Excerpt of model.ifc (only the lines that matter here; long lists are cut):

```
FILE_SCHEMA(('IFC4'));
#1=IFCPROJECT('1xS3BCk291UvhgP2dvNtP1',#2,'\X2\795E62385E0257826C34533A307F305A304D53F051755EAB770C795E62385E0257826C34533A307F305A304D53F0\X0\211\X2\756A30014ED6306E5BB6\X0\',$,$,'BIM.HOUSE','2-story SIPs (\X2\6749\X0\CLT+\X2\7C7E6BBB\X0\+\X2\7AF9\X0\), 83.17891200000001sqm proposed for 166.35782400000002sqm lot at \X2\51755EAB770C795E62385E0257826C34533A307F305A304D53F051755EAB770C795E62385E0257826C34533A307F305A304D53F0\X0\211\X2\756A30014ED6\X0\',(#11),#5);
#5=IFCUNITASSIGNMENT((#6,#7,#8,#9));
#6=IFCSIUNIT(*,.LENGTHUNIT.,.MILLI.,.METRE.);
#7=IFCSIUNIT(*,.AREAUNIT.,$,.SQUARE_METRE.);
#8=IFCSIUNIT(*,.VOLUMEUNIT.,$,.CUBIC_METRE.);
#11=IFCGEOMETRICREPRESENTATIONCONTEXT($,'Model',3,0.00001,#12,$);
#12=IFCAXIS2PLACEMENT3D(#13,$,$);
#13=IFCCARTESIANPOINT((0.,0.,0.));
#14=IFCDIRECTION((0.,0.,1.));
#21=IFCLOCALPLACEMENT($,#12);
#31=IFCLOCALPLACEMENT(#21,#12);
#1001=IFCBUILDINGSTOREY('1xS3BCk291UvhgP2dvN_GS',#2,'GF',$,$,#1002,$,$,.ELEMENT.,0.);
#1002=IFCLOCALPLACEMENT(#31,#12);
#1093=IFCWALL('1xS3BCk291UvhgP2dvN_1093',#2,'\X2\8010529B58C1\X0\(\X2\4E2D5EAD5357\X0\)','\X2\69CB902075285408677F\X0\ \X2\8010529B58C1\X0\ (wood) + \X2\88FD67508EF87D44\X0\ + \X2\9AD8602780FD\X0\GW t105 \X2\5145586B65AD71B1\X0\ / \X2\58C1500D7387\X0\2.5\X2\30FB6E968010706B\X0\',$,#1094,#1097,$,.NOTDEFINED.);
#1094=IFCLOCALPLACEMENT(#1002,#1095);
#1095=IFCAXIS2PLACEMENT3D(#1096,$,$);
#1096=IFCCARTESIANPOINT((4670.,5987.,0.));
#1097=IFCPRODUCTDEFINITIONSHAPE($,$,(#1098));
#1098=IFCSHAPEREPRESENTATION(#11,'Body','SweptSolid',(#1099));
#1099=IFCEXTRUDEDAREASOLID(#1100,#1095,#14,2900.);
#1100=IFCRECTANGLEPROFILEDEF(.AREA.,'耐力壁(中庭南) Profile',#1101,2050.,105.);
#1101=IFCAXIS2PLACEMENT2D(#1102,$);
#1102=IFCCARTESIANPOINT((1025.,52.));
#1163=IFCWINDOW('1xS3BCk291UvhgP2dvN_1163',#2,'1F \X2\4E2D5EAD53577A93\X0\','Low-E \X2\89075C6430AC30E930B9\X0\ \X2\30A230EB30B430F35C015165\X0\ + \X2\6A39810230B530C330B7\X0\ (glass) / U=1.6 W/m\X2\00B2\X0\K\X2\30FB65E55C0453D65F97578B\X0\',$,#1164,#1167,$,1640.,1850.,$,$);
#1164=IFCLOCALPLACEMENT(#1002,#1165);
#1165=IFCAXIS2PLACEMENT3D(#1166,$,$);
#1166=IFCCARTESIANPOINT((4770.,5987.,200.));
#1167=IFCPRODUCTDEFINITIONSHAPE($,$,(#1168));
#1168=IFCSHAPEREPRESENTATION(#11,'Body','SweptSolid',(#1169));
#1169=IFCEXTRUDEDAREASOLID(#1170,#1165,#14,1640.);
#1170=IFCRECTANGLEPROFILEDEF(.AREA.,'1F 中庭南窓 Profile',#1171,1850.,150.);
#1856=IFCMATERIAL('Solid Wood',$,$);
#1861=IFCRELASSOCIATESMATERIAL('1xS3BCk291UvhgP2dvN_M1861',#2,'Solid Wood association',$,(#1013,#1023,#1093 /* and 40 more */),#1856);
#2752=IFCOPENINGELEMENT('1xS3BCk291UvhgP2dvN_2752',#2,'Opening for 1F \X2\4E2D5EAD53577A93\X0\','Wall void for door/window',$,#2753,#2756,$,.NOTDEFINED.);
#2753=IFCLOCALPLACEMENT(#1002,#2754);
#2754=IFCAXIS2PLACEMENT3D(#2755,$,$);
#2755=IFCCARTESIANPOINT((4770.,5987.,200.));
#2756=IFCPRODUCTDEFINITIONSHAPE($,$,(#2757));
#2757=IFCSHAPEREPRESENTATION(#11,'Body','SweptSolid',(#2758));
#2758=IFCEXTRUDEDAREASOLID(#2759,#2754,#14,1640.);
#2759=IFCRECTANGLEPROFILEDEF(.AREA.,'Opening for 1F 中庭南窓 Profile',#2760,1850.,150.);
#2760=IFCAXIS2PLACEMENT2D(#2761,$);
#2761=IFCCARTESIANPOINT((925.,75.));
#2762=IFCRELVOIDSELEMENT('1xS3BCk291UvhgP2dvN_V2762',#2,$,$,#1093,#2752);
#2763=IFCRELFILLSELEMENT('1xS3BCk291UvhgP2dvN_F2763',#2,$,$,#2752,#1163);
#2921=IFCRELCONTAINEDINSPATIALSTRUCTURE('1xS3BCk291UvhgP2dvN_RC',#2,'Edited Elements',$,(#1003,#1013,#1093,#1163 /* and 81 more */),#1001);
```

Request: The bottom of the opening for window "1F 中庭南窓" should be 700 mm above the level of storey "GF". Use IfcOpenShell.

```python
import numpy as np
import ifcopenshell
import ifcopenshell.api.geometry
import ifcopenshell.geom
import ifcopenshell.util.element
import ifcopenshell.util.placement
import ifcopenshell.util.shape
import ifcopenshell.util.unit

model = ifcopenshell.open("model.ifc")
unit_scale = ifcopenshell.util.unit.calculate_unit_scale(model)

window = model.by_guid("1xS3BCk291UvhgP2dvN_1163")
opening = window.FillsVoids[0].RelatingOpeningElement
storey = ifcopenshell.util.element.get_container(window, ifc_class="IfcBuildingStorey")
level = ifcopenshell.util.placement.get_local_placement(storey.ObjectPlacement)[2, 3]

# The opening's origin need not be at the sill, so measure its lowest point.
shape = ifcopenshell.geom.create_shape(ifcopenshell.geom.settings(), opening)
bottom = ifcopenshell.util.shape.get_shape_bottom_elevation(shape, shape.geometry) / unit_scale
dz = level + 0.7 / unit_scale - bottom

shift = np.array([0.0, 0.0, dz])
# The window is not placed relative to its opening, so move both.
for product in (opening, window):
    matrix = ifcopenshell.util.placement.get_local_placement(product.ObjectPlacement)
    matrix[:3, 3] += shift
    ifcopenshell.api.geometry.edit_object_placement(model, product=product, matrix=matrix, is_si=False)

print(f"moved by {dz * unit_scale:+.3f} m")

model.write("model_updated.ifc")
```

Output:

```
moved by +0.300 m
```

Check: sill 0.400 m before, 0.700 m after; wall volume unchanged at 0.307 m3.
